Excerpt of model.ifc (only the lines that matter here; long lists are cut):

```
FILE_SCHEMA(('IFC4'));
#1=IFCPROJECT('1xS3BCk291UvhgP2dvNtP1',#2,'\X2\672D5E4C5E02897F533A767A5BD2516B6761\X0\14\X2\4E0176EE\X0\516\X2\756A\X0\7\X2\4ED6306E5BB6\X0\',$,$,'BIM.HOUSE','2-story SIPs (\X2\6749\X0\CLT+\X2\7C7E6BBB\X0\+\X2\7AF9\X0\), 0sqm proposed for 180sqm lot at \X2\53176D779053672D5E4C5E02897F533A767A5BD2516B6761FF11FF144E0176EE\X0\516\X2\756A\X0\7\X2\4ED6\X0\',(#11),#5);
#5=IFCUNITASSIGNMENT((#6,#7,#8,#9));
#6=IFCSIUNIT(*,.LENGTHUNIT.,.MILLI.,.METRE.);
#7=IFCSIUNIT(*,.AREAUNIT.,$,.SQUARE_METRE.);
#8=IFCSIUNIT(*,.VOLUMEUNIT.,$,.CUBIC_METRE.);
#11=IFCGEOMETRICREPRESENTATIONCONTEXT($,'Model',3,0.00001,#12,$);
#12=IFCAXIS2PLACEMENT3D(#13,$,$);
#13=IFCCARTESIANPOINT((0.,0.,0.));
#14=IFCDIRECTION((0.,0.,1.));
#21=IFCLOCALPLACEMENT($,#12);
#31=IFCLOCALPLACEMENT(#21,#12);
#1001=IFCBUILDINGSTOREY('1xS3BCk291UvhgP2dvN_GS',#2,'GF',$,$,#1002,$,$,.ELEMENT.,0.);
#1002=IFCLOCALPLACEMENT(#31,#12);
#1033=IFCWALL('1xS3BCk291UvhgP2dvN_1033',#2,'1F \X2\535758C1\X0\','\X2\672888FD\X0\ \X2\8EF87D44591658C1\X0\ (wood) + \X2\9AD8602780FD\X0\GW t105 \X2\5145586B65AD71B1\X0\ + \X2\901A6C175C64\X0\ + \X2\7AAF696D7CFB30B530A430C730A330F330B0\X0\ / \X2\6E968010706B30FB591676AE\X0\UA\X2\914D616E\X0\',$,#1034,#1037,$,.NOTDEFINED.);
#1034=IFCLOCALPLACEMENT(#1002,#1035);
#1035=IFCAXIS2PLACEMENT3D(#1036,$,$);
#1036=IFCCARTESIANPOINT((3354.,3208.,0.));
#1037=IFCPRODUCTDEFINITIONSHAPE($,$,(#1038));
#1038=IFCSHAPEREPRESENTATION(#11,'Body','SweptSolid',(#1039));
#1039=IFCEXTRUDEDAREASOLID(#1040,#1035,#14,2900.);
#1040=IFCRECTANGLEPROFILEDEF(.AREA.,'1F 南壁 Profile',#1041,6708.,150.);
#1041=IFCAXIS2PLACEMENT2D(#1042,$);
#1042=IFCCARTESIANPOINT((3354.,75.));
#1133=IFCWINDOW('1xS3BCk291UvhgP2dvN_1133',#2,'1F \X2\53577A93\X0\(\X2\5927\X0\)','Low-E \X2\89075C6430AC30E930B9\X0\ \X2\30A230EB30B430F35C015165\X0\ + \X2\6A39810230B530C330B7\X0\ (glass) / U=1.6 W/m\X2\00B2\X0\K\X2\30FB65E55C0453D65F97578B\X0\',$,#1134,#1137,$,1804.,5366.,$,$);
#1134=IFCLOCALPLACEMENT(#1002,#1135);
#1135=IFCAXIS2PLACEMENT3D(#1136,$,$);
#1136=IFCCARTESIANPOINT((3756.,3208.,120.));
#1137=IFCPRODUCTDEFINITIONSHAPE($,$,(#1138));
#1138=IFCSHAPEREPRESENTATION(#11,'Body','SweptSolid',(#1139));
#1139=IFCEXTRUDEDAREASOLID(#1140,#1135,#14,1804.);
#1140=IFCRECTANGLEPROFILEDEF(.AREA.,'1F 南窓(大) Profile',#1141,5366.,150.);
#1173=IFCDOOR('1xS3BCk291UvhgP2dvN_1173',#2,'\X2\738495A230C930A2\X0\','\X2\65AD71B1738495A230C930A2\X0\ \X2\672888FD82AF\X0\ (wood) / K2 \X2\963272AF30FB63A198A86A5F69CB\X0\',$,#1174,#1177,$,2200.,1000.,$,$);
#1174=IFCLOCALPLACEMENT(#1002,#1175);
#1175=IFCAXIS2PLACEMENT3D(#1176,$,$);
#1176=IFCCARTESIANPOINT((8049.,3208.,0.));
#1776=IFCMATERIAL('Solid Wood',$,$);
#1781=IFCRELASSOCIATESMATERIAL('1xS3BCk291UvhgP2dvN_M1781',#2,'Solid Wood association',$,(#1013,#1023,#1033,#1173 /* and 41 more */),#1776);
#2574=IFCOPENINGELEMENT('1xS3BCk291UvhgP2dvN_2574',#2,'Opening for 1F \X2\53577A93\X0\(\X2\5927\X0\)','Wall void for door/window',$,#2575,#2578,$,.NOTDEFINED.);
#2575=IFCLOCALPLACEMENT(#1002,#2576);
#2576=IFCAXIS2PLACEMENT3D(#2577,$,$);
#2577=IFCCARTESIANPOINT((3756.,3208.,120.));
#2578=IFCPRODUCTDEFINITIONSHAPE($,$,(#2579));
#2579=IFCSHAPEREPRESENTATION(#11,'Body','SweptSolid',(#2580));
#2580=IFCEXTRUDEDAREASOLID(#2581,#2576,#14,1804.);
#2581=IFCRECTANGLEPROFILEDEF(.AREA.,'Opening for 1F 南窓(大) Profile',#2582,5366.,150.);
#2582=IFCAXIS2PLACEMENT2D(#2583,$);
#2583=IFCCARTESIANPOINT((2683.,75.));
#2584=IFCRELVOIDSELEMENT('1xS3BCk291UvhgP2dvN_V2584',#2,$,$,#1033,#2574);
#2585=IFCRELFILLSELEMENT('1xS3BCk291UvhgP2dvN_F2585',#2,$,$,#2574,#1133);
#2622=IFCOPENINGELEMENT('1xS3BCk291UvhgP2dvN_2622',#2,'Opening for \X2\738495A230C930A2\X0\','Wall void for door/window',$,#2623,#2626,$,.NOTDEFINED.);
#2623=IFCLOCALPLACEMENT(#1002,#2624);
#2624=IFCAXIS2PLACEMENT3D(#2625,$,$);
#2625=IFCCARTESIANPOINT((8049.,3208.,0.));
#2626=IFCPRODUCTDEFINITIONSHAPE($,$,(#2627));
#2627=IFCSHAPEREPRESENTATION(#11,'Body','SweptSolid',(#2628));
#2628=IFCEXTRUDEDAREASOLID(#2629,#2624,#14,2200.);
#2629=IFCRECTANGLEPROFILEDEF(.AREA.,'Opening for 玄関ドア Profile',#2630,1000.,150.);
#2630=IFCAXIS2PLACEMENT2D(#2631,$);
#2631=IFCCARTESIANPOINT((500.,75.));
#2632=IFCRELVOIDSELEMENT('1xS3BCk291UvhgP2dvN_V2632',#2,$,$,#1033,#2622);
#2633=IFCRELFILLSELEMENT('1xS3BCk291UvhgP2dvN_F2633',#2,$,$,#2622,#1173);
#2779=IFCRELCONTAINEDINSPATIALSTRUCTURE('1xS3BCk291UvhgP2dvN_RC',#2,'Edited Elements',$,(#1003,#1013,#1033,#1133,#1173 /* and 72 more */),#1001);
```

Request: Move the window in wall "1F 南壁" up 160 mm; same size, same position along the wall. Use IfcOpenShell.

```python
import numpy as np
import ifcopenshell
import ifcopenshell.api.geometry
import ifcopenshell.util.placement
import ifcopenshell.util.unit

model = ifcopenshell.open("model.ifc")
unit_scale = ifcopenshell.util.unit.calculate_unit_scale(model)

window = model.by_guid("1xS3BCk291UvhgP2dvN_1133")
opening = window.FillsVoids[0].RelatingOpeningElement
dz = 0.16 / unit_scale

shift = np.array([0.0, 0.0, dz])
# The window is not placed relative to its opening, so move both.
for product in (opening, window):
    matrix = ifcopenshell.util.placement.get_local_placement(product.ObjectPlacement)
    matrix[:3, 3] += shift
    ifcopenshell.api.geometry.edit_object_placement(model, product=product, matrix=matrix, is_si=False)

print(f"moved by {dz * unit_scale:+.3f} m")

model.write("model_edited.ifc")
```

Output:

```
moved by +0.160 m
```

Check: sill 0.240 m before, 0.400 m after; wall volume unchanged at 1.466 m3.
